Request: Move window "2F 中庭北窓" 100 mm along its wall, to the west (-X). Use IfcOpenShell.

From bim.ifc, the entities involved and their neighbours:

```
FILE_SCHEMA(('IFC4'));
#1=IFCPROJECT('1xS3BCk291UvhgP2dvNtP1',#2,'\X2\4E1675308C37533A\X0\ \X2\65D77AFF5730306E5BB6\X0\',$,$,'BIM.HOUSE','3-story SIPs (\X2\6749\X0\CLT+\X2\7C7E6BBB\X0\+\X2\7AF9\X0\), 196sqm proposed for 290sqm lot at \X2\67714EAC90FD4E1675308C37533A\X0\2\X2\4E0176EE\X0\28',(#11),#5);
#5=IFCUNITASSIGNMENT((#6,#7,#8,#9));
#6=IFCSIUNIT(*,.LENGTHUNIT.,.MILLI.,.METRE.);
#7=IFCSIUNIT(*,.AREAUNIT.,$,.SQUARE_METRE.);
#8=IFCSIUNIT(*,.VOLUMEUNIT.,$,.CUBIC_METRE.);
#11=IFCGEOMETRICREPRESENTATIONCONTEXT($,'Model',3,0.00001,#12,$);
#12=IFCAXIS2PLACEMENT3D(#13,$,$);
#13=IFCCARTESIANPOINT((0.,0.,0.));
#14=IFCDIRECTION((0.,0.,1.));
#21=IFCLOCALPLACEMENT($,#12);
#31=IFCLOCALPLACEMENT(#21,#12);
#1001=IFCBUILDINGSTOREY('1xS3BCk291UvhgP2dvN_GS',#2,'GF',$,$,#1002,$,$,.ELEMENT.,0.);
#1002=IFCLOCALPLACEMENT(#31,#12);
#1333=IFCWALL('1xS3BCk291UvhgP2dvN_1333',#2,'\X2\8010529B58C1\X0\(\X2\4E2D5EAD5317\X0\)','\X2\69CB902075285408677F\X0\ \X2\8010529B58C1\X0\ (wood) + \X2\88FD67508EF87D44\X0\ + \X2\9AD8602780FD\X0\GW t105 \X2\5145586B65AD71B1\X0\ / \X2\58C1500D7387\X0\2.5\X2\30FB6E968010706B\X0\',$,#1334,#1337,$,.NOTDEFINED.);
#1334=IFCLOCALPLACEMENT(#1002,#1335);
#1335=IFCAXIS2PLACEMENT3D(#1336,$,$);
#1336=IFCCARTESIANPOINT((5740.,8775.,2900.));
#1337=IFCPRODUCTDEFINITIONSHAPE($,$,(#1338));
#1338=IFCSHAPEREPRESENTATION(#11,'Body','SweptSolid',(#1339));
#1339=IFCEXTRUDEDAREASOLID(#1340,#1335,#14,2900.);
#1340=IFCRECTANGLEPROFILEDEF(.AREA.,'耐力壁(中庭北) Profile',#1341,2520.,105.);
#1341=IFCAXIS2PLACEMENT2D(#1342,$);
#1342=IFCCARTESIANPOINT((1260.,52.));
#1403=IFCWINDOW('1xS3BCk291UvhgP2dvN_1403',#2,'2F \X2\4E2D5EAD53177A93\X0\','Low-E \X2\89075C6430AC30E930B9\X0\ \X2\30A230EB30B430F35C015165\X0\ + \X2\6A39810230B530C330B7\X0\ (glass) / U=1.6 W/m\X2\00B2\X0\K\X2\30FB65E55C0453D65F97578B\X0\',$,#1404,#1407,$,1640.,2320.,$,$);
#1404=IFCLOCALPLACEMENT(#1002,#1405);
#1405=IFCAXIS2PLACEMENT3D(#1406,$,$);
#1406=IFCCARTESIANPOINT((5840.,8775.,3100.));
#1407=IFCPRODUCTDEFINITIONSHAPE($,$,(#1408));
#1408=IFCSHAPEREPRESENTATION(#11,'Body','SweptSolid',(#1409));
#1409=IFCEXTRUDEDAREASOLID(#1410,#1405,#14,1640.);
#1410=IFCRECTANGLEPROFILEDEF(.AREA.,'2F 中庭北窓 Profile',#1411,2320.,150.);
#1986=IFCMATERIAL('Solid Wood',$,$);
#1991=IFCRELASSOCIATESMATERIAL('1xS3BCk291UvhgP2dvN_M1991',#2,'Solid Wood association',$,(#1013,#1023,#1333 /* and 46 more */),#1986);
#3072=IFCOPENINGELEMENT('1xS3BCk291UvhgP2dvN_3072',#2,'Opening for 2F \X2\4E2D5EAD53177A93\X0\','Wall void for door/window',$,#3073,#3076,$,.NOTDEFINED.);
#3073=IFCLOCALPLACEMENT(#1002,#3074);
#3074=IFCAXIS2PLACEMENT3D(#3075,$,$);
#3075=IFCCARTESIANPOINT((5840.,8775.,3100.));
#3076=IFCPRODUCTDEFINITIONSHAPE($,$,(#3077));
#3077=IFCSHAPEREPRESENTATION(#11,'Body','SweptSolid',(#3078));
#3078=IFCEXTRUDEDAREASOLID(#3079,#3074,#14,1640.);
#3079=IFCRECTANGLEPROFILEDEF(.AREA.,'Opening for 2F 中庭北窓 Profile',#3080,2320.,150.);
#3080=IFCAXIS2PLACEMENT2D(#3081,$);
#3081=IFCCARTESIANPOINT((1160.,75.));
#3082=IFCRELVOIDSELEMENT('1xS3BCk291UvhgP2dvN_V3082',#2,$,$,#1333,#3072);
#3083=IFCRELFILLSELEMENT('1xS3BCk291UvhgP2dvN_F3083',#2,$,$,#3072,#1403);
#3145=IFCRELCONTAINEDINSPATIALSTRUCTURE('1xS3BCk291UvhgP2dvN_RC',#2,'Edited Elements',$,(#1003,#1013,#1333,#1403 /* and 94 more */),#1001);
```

```python
import ifcopenshell
import ifcopenshell.api.geometry
import ifcopenshell.util.placement
import ifcopenshell.util.unit

model = ifcopenshell.open("bim.ifc")
unit_scale = ifcopenshell.util.unit.calculate_unit_scale(model)

window = model.by_guid("1xS3BCk291UvhgP2dvN_1403")
opening = window.FillsVoids[0].RelatingOpeningElement
wall = opening.VoidsElements[0].RelatingBuildingElement

wall_matrix = ifcopenshell.util.placement.get_local_placement(wall.ObjectPlacement)
shift = wall_matrix[:3, 0] * -0.1 / unit_scale
before = ifcopenshell.util.placement.get_local_placement(window.ObjectPlacement)[:3, 3].copy()

# The window is not placed relative to its opening, so move both.
for product in (opening, window):
    matrix = ifcopenshell.util.placement.get_local_placement(product.ObjectPlacement)
    matrix[:3, 3] += shift
    ifcopenshell.api.geometry.edit_object_placement(model, product=product, matrix=matrix, is_si=False)

after = ifcopenshell.util.placement.get_local_placement(window.ObjectPlacement)[:3, 3]
print("window moved by", (after - before).round(3) + 0.0)

model.write("bim_rev.ifc")
```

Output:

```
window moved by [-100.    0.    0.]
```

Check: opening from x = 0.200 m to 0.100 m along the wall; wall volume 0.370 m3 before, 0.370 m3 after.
